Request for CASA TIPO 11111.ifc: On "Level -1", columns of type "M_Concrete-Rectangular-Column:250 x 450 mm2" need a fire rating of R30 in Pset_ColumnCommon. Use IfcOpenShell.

First a look at what the model holds.

```python
import ifcopenshell
import ifcopenshell.util.element

model = ifcopenshell.open("CASA TIPO 11111.ifc")
print(model.schema)
storey = next(s for s in model.by_type("IfcBuildingStorey") if s.Name == "Level -1")
columns = [e for e in ifcopenshell.util.element.get_decomposition(storey) if e.is_a("IfcColumn")]
seen = {}
for e in columns:
    element_type = ifcopenshell.util.element.get_type(e)
    key = (element_type.Name if element_type != e and element_type else None, ifcopenshell.util.element.get_pset(e, "Pset_ColumnCommon", "FireRating"))
    seen[key] = seen.get(key, 0) + 1
for (name, value), count in sorted(seen.items(), key=str):
    print(count, "x", name, "|", value)
```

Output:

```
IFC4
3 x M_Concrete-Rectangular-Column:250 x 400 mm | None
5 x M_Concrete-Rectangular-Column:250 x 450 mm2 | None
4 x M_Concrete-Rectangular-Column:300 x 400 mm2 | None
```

```python
import ifcopenshell
import ifcopenshell.api.pset
import ifcopenshell.util.element

model = ifcopenshell.open("CASA TIPO 11111.ifc")

storey = next(s for s in model.by_type("IfcBuildingStorey") if s.Name == "Level -1")
columns = [e for e in ifcopenshell.util.element.get_decomposition(storey) if e.is_a("IfcColumn")]

count = 0
for e in columns:
    element_type = ifcopenshell.util.element.get_type(e)
    if element_type in (None, e) or element_type.Name != "M_Concrete-Rectangular-Column:250 x 450 mm2":
        continue
    # add_pset returns the element's existing set when there is one.
    pset = ifcopenshell.api.pset.add_pset(model, product=e, name="Pset_ColumnCommon")
    ifcopenshell.api.pset.edit_pset(model, pset=pset, properties={"FireRating": "R30"})
    count += 1

print(count, "columns updated")

model.write("CASA TIPO 11111_rev.ifc")
```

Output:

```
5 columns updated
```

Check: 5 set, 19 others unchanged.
